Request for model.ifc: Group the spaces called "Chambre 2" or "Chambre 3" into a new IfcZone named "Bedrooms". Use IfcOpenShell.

First a look at what the model holds.

```python
import ifcopenshell

model = ifcopenshell.open("model.ifc")
print(model.schema)
seen = {}
for space in model.by_type("IfcSpace"):
    seen[space.LongName] = seen.get(space.LongName, 0) + 1
for name, count in sorted(seen.items(), key=str):
    print(count, "x", name)
print("zones:", [z.Name for z in model.by_type("IfcZone")][:20])
```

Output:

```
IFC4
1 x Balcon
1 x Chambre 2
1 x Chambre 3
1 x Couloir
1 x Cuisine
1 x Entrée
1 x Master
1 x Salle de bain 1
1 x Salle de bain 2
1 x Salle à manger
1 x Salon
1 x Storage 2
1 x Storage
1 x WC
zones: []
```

```python
import ifcopenshell
import ifcopenshell.api.group
import ifcopenshell.api.root

model = ifcopenshell.open("model.ifc")

names = {"Chambre 2", "Chambre 3"}
spaces = [s for s in model.by_type("IfcSpace") if s.LongName in names]

zone = ifcopenshell.api.root.create_entity(model, ifc_class="IfcZone", name="Bedrooms")
ifcopenshell.api.group.assign_group(model, products=spaces, group=zone)
print(len(spaces), "spaces in", zone.Name)

model.write("model-out.ifc")
```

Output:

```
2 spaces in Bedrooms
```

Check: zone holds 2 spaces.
